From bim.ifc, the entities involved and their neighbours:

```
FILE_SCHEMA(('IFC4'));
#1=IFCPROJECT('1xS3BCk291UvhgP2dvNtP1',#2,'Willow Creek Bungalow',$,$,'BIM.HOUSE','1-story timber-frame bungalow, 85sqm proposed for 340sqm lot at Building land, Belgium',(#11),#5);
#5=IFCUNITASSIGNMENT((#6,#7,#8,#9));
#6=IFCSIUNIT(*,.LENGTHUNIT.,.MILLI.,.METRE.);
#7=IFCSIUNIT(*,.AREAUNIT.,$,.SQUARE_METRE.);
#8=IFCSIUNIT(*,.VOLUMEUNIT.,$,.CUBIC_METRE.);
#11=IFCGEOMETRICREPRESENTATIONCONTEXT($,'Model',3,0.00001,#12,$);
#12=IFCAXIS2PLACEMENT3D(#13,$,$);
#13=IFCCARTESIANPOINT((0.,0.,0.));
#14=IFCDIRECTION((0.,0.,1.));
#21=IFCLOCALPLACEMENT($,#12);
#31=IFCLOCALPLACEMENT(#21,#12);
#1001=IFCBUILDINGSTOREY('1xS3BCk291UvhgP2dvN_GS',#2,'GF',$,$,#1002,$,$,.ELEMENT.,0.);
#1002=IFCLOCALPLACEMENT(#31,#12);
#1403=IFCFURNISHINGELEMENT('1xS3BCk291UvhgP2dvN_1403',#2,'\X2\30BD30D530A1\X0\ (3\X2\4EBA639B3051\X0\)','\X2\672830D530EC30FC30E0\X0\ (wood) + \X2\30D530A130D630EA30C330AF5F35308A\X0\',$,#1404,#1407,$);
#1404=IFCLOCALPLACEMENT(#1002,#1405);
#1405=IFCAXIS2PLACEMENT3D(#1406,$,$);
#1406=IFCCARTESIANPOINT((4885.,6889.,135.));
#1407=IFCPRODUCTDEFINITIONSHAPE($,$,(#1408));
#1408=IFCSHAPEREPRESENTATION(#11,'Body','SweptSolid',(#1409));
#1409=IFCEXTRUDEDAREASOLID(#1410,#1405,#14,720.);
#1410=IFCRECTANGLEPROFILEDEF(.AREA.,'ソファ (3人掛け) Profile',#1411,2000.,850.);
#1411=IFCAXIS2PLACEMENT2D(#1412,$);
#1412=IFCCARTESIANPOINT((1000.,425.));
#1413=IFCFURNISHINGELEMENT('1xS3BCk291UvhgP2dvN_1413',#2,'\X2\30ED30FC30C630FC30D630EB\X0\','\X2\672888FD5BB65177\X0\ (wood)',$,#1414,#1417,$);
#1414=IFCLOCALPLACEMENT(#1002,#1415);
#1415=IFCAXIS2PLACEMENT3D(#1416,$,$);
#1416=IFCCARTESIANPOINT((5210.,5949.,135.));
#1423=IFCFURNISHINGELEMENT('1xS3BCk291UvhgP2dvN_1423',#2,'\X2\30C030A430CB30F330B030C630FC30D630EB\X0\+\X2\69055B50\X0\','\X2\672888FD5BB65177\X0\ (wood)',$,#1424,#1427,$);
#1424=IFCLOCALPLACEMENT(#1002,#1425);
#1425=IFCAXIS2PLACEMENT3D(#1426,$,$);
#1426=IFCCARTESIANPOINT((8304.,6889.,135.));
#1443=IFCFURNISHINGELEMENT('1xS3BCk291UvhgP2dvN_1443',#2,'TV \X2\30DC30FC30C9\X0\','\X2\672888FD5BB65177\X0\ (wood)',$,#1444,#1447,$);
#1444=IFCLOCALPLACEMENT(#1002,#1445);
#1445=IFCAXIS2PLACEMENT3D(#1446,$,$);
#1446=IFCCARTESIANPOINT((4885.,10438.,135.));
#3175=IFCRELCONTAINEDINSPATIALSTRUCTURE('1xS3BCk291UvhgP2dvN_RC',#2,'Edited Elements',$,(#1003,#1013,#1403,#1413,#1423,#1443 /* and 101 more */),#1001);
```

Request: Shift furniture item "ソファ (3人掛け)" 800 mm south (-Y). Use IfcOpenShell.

```python
import ifcopenshell
import ifcopenshell.api.geometry
import ifcopenshell.util.placement
import ifcopenshell.util.unit

model = ifcopenshell.open("bim.ifc")
unit_scale = ifcopenshell.util.unit.calculate_unit_scale(model)

item = model.by_id(1403)
matrix = ifcopenshell.util.placement.get_local_placement(item.ObjectPlacement)
matrix[1, 3] -= 0.8 / unit_scale
ifcopenshell.api.geometry.edit_object_placement(model, product=item, matrix=matrix, is_si=False)

print(ifcopenshell.util.placement.get_local_placement(item.ObjectPlacement).round(3) + 0.0)

model.write("bim_edited.ifc")
```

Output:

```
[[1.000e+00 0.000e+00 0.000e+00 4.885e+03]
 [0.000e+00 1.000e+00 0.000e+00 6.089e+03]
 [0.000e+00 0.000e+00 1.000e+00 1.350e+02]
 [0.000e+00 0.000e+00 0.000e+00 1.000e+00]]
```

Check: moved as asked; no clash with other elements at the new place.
